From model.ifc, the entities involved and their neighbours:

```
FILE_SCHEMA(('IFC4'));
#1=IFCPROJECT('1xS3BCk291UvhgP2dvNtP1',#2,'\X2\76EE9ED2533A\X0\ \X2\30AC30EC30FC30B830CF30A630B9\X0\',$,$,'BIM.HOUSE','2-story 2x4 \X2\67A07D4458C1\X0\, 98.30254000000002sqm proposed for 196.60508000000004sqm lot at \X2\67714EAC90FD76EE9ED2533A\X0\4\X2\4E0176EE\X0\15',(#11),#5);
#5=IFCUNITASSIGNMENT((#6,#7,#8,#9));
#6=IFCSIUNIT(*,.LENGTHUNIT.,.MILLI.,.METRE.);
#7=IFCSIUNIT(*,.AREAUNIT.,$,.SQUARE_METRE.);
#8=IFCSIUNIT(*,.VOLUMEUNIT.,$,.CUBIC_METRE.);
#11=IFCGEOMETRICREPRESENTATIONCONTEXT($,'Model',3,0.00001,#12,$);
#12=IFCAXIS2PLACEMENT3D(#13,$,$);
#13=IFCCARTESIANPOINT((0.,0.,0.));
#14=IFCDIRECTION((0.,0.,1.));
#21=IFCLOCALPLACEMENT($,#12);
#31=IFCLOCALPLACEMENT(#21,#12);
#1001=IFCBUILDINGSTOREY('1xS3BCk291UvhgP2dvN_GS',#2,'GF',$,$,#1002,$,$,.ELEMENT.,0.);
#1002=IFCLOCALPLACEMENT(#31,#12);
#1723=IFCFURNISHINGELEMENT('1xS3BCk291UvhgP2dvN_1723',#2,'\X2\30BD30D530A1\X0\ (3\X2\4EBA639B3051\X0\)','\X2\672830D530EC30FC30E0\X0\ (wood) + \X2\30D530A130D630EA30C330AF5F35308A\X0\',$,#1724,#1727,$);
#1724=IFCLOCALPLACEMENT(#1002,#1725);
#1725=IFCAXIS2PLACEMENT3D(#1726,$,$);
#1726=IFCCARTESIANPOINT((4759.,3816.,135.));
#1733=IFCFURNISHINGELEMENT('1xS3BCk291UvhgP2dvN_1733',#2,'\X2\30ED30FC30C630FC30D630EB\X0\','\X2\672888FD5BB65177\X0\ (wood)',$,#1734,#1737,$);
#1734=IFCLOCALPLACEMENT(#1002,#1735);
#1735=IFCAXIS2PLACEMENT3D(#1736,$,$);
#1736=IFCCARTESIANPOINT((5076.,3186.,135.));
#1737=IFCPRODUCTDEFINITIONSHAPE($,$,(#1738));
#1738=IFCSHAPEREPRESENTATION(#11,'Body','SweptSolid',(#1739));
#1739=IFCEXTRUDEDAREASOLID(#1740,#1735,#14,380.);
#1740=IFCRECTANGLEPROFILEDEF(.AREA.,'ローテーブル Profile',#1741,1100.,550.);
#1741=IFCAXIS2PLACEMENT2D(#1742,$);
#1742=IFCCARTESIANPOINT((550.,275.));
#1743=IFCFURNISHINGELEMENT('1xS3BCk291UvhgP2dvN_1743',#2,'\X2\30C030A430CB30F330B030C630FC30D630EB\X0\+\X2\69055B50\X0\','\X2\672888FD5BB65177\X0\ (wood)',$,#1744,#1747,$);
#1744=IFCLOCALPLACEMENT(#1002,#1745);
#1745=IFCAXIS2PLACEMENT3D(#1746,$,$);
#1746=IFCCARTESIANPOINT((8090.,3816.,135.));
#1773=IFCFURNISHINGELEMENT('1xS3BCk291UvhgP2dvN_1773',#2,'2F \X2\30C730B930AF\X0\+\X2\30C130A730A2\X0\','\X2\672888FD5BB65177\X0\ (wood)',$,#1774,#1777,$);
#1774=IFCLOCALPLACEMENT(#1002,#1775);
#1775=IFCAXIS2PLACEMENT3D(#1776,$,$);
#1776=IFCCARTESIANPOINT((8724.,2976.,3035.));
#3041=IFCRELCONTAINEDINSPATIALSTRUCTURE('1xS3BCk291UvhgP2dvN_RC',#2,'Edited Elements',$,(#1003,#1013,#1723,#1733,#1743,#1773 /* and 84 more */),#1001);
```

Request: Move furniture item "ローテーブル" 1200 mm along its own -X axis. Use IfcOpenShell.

```python
import ifcopenshell
import ifcopenshell.api.geometry
import ifcopenshell.util.placement
import ifcopenshell.util.unit

model = ifcopenshell.open("model.ifc")
unit_scale = ifcopenshell.util.unit.calculate_unit_scale(model)

item = model.by_guid("1xS3BCk291UvhgP2dvN_1733")
matrix = ifcopenshell.util.placement.get_local_placement(item.ObjectPlacement)
matrix[:3, 3] -= matrix[:3, 0] * 1.2 / unit_scale
ifcopenshell.api.geometry.edit_object_placement(model, product=item, matrix=matrix, is_si=False)

print(ifcopenshell.util.placement.get_local_placement(item.ObjectPlacement).round(3) + 0.0)

model.write("model_edited.ifc")
```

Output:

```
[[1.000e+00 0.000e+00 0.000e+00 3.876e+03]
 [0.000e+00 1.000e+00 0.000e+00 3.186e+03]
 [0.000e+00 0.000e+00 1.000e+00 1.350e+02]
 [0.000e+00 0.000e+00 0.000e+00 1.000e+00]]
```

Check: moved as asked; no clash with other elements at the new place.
